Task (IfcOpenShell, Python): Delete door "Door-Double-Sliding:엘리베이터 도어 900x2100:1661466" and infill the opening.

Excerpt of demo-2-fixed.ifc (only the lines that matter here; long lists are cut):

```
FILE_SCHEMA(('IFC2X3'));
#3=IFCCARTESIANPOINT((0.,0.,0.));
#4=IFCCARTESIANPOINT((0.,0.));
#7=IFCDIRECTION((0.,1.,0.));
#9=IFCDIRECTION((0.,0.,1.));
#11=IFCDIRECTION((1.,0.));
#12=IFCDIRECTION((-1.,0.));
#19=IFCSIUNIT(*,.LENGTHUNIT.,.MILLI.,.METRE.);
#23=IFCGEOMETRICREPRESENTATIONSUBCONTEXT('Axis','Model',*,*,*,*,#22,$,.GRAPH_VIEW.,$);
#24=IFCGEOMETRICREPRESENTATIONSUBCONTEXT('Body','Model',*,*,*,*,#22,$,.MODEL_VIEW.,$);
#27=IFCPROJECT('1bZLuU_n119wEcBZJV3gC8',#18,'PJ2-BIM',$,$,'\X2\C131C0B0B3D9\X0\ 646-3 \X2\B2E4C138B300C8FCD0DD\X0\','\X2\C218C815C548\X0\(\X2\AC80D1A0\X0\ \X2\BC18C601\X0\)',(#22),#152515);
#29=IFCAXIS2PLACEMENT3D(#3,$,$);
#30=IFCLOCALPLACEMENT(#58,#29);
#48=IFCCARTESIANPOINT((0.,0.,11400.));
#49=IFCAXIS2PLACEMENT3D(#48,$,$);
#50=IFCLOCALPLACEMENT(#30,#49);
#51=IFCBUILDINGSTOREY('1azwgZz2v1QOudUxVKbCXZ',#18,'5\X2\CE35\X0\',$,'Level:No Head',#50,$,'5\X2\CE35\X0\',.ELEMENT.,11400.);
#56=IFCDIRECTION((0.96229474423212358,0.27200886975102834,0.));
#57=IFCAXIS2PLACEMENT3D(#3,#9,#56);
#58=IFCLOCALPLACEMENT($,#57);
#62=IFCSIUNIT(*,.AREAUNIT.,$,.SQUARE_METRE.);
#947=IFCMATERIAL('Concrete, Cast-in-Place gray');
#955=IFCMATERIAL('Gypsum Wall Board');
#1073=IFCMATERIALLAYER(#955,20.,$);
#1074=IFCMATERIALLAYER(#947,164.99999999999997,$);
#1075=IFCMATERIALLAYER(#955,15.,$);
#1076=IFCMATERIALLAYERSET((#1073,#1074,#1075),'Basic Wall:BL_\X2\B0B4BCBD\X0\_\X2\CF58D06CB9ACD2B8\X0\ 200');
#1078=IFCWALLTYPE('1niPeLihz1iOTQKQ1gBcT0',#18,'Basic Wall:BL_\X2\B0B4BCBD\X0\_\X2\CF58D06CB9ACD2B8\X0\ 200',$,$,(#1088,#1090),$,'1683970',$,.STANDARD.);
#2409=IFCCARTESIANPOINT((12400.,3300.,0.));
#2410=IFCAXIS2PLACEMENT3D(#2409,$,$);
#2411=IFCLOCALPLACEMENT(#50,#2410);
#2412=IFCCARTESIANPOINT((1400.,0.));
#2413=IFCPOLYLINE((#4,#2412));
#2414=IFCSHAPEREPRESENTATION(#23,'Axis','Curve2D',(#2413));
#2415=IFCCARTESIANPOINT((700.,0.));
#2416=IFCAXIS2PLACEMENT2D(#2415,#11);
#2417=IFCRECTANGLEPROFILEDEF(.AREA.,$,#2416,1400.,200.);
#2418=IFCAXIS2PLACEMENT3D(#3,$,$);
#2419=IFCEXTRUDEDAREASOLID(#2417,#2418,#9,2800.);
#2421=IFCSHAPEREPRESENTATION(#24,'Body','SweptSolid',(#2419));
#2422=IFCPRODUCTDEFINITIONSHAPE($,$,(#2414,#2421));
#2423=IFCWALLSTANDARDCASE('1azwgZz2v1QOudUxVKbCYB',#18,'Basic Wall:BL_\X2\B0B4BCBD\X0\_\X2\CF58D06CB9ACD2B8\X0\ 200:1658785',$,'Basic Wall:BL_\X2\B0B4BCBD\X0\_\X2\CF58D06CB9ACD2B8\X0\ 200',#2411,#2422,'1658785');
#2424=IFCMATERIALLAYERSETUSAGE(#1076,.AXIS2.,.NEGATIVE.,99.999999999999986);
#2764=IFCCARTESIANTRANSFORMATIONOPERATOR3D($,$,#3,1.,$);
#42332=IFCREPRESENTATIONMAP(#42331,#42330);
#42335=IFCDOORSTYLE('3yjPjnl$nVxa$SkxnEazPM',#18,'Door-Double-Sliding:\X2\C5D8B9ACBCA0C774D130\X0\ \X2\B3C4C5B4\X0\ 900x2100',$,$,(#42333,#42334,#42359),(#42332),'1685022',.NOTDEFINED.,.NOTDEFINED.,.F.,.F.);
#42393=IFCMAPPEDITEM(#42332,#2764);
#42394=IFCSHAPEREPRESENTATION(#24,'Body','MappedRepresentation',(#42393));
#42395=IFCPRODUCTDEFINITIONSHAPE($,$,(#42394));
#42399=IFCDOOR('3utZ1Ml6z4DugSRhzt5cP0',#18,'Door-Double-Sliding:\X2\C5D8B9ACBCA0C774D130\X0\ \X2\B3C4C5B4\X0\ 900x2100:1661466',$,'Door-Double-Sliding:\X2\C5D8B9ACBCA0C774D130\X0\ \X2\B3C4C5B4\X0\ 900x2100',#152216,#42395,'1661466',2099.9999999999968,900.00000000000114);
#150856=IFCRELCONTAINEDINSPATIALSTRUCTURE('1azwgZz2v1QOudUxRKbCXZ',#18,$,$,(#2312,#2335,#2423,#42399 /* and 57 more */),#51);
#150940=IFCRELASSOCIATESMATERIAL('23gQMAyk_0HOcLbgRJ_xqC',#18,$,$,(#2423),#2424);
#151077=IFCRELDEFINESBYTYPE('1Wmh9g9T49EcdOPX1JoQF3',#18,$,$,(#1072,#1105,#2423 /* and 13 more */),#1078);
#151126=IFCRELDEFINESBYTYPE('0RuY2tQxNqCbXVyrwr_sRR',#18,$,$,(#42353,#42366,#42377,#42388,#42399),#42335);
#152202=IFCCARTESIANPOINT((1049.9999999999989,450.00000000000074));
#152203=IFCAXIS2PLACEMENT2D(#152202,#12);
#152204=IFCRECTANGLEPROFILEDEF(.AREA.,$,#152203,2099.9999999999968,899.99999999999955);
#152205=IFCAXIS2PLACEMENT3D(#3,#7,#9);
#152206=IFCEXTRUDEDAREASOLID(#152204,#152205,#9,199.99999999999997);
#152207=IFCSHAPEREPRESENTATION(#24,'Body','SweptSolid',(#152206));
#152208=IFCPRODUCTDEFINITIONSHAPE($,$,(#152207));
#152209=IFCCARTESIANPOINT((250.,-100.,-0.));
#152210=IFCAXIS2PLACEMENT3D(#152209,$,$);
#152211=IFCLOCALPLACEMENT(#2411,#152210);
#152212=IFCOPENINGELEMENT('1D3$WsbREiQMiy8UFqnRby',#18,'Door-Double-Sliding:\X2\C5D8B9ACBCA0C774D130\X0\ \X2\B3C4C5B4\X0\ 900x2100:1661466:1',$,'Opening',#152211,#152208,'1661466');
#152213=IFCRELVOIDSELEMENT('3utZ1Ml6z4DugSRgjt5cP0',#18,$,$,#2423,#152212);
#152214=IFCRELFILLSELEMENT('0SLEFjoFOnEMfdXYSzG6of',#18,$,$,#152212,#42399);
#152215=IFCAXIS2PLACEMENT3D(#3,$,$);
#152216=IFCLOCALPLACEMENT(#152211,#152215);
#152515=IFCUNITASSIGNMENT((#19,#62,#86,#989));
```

```python
import ifcopenshell
import ifcopenshell.api.feature
import ifcopenshell.api.root
import ifcopenshell.geom
import ifcopenshell.util.shape

model = ifcopenshell.open("demo-2-fixed.ifc")
settings = ifcopenshell.geom.settings()


def volume(element):
    """Net volume in cubic metres, openings subtracted."""
    shape = ifcopenshell.geom.create_shape(settings, element)
    return ifcopenshell.util.shape.get_volume(shape.geometry)


door = model.by_guid("3utZ1Ml6z4DugSRhzt5cP0")
opening = door.FillsVoids[0].RelatingOpeningElement
wall = opening.VoidsElements[0].RelatingBuildingElement
before = volume(wall)

ifcopenshell.api.root.remove_product(model, product=door)
ifcopenshell.api.feature.remove_feature(model, feature=opening)

after = volume(wall)

print(f"wall volume {before:.3f} -> {after:.3f} m3")

model.write("demo-2-fixed_updated.ifc")
```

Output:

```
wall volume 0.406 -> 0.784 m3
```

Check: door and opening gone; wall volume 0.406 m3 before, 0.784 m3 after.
